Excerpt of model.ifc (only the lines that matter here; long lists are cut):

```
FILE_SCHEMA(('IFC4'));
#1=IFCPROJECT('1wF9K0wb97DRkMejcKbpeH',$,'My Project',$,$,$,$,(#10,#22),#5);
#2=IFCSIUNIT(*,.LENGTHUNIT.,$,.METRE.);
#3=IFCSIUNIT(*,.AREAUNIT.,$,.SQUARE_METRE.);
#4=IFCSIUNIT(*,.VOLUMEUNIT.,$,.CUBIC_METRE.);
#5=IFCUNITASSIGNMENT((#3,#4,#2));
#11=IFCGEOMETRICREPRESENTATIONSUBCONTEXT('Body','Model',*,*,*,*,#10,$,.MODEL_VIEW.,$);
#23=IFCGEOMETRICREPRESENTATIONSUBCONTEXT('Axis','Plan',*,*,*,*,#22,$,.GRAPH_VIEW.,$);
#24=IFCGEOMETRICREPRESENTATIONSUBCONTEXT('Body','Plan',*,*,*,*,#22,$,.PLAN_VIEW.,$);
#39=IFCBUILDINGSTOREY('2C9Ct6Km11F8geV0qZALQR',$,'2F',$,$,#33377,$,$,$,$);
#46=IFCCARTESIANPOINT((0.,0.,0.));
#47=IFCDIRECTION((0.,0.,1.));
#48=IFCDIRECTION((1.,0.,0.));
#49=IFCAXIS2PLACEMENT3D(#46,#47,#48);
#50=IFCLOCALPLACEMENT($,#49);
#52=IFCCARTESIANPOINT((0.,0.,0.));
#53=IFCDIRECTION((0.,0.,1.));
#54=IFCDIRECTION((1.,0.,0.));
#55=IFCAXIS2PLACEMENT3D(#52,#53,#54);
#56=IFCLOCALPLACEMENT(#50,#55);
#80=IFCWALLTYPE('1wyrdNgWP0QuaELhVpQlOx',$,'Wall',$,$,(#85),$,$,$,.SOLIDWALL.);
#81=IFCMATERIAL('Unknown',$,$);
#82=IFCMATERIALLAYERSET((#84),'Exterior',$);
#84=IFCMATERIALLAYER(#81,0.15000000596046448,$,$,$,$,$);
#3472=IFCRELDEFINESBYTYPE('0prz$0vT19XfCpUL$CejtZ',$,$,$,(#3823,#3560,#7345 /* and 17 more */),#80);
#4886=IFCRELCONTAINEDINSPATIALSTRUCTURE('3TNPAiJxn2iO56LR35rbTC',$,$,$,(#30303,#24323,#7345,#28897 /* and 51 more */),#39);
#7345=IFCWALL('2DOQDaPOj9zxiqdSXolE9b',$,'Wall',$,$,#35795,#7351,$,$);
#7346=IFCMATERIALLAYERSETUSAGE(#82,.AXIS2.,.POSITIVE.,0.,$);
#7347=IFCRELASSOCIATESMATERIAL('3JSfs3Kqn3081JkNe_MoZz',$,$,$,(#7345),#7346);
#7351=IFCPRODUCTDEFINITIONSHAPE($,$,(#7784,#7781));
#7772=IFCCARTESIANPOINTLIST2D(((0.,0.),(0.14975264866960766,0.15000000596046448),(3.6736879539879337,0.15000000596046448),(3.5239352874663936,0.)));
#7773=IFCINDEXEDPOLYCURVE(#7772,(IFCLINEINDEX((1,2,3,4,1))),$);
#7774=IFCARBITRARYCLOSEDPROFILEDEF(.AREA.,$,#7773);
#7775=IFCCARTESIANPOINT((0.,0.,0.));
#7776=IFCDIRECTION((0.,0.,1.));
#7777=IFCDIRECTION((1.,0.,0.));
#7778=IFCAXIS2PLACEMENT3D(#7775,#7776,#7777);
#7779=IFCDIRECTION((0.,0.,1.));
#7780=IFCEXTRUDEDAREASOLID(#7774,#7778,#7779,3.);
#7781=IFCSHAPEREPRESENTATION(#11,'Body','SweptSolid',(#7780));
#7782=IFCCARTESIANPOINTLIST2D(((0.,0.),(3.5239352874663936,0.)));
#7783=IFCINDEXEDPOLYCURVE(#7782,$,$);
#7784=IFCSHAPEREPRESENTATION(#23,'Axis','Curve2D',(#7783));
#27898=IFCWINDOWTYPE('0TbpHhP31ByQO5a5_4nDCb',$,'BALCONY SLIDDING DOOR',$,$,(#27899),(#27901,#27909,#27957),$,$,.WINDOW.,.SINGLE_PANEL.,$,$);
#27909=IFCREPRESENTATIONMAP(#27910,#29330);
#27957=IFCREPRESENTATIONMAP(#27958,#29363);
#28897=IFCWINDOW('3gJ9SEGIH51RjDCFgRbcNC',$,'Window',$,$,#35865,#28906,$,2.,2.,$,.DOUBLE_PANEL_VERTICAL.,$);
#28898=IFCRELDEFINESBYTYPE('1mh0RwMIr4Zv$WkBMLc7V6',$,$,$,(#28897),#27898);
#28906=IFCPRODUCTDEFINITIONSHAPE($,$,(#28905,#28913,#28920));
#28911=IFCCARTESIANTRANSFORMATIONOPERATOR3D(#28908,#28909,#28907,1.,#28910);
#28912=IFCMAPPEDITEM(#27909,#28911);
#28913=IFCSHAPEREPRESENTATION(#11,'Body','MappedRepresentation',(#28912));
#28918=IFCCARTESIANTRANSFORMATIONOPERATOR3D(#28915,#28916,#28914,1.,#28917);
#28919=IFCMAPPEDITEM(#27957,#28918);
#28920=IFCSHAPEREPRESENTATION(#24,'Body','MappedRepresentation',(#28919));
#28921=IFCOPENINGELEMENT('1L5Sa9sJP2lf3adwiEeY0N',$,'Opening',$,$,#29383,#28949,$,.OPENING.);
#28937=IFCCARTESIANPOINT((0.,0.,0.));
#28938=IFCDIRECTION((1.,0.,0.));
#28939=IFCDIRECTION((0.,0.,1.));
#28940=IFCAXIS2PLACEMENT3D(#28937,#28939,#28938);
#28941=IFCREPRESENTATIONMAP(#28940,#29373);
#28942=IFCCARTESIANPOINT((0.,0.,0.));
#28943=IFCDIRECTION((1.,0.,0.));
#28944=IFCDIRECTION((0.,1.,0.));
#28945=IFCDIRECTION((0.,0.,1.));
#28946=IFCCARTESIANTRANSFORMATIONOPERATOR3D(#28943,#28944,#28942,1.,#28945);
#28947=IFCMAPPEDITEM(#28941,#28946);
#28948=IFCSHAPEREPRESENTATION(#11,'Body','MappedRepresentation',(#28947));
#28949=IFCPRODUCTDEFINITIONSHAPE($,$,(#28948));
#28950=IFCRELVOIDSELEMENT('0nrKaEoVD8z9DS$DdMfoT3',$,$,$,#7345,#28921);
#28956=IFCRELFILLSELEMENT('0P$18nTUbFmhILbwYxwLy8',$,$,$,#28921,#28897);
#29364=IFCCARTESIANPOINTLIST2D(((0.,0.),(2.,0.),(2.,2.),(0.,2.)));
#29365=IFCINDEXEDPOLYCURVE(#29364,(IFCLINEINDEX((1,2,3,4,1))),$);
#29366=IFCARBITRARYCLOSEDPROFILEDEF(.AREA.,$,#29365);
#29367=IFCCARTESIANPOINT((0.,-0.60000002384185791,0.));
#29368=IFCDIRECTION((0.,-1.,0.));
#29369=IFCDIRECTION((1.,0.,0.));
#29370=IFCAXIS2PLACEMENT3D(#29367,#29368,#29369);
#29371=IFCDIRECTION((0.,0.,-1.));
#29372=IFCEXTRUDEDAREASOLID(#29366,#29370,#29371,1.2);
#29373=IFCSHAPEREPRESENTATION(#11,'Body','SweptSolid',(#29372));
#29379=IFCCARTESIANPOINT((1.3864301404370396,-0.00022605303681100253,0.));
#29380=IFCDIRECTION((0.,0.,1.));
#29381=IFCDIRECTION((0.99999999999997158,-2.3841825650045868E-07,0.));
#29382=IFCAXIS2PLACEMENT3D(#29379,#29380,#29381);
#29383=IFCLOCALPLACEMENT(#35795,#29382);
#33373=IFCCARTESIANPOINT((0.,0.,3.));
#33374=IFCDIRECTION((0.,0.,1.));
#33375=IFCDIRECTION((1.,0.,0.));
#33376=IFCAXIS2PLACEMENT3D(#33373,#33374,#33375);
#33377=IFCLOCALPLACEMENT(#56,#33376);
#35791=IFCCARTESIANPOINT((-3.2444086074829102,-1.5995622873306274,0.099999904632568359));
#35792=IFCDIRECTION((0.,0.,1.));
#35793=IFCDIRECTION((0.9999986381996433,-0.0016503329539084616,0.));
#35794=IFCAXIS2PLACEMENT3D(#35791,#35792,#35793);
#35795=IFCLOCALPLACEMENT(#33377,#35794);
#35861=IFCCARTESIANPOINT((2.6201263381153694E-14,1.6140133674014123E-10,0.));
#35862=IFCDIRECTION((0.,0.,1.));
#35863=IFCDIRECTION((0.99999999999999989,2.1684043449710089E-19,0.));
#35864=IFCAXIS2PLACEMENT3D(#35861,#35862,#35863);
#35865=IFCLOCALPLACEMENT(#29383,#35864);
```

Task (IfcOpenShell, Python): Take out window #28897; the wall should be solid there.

```python
import ifcopenshell
import ifcopenshell.api.feature
import ifcopenshell.api.root
import ifcopenshell.geom
import ifcopenshell.util.shape

model = ifcopenshell.open("model.ifc")
settings = ifcopenshell.geom.settings()


def volume(element):
    """Net volume in cubic metres, openings subtracted."""
    shape = ifcopenshell.geom.create_shape(settings, element)
    return ifcopenshell.util.shape.get_volume(shape.geometry)


window = model.by_id(28897)
opening = window.FillsVoids[0].RelatingOpeningElement
wall = opening.VoidsElements[0].RelatingBuildingElement
before = volume(wall)

ifcopenshell.api.root.remove_product(model, product=window)
ifcopenshell.api.feature.remove_feature(model, feature=opening)

after = volume(wall)

print(f"wall volume {before:.3f} -> {after:.3f} m3")

model.write("model_v2.ifc")
```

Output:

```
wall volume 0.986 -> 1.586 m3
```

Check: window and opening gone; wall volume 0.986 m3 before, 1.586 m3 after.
